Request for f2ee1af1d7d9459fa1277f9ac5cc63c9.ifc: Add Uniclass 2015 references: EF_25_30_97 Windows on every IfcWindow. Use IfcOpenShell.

First a look at what the model holds.

```python
import ifcopenshell

model = ifcopenshell.open("f2ee1af1d7d9459fa1277f9ac5cc63c9.ifc")
print(model.schema)
print("classifications:", [c.Name for c in model.by_type("IfcClassification")])
for ifc_class in ("IfcDoor", "IfcRoof", "IfcStair", "IfcWall", "IfcWindow"):
    print(ifc_class, len(model.by_type(ifc_class)))
```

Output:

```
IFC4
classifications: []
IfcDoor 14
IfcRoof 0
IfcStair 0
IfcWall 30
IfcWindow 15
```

```python
import ifcopenshell
import ifcopenshell.api.classification

model = ifcopenshell.open("f2ee1af1d7d9459fa1277f9ac5cc63c9.ifc")

system = ifcopenshell.api.classification.add_classification(model, classification="Uniclass 2015")

codes = {
    "IfcWindow": ("EF_25_30_97", "Windows"),
}
for ifc_class, (code, name) in codes.items():
    products = model.by_type(ifc_class)
    ifcopenshell.api.classification.add_reference(
        model, products=products, classification=system, identification=code, name=name
    )
    print(code, len(products))

model.write("f2ee1af1d7d9459fa1277f9ac5cc63c9_edited.ifc")
```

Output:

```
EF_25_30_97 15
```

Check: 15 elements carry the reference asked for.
